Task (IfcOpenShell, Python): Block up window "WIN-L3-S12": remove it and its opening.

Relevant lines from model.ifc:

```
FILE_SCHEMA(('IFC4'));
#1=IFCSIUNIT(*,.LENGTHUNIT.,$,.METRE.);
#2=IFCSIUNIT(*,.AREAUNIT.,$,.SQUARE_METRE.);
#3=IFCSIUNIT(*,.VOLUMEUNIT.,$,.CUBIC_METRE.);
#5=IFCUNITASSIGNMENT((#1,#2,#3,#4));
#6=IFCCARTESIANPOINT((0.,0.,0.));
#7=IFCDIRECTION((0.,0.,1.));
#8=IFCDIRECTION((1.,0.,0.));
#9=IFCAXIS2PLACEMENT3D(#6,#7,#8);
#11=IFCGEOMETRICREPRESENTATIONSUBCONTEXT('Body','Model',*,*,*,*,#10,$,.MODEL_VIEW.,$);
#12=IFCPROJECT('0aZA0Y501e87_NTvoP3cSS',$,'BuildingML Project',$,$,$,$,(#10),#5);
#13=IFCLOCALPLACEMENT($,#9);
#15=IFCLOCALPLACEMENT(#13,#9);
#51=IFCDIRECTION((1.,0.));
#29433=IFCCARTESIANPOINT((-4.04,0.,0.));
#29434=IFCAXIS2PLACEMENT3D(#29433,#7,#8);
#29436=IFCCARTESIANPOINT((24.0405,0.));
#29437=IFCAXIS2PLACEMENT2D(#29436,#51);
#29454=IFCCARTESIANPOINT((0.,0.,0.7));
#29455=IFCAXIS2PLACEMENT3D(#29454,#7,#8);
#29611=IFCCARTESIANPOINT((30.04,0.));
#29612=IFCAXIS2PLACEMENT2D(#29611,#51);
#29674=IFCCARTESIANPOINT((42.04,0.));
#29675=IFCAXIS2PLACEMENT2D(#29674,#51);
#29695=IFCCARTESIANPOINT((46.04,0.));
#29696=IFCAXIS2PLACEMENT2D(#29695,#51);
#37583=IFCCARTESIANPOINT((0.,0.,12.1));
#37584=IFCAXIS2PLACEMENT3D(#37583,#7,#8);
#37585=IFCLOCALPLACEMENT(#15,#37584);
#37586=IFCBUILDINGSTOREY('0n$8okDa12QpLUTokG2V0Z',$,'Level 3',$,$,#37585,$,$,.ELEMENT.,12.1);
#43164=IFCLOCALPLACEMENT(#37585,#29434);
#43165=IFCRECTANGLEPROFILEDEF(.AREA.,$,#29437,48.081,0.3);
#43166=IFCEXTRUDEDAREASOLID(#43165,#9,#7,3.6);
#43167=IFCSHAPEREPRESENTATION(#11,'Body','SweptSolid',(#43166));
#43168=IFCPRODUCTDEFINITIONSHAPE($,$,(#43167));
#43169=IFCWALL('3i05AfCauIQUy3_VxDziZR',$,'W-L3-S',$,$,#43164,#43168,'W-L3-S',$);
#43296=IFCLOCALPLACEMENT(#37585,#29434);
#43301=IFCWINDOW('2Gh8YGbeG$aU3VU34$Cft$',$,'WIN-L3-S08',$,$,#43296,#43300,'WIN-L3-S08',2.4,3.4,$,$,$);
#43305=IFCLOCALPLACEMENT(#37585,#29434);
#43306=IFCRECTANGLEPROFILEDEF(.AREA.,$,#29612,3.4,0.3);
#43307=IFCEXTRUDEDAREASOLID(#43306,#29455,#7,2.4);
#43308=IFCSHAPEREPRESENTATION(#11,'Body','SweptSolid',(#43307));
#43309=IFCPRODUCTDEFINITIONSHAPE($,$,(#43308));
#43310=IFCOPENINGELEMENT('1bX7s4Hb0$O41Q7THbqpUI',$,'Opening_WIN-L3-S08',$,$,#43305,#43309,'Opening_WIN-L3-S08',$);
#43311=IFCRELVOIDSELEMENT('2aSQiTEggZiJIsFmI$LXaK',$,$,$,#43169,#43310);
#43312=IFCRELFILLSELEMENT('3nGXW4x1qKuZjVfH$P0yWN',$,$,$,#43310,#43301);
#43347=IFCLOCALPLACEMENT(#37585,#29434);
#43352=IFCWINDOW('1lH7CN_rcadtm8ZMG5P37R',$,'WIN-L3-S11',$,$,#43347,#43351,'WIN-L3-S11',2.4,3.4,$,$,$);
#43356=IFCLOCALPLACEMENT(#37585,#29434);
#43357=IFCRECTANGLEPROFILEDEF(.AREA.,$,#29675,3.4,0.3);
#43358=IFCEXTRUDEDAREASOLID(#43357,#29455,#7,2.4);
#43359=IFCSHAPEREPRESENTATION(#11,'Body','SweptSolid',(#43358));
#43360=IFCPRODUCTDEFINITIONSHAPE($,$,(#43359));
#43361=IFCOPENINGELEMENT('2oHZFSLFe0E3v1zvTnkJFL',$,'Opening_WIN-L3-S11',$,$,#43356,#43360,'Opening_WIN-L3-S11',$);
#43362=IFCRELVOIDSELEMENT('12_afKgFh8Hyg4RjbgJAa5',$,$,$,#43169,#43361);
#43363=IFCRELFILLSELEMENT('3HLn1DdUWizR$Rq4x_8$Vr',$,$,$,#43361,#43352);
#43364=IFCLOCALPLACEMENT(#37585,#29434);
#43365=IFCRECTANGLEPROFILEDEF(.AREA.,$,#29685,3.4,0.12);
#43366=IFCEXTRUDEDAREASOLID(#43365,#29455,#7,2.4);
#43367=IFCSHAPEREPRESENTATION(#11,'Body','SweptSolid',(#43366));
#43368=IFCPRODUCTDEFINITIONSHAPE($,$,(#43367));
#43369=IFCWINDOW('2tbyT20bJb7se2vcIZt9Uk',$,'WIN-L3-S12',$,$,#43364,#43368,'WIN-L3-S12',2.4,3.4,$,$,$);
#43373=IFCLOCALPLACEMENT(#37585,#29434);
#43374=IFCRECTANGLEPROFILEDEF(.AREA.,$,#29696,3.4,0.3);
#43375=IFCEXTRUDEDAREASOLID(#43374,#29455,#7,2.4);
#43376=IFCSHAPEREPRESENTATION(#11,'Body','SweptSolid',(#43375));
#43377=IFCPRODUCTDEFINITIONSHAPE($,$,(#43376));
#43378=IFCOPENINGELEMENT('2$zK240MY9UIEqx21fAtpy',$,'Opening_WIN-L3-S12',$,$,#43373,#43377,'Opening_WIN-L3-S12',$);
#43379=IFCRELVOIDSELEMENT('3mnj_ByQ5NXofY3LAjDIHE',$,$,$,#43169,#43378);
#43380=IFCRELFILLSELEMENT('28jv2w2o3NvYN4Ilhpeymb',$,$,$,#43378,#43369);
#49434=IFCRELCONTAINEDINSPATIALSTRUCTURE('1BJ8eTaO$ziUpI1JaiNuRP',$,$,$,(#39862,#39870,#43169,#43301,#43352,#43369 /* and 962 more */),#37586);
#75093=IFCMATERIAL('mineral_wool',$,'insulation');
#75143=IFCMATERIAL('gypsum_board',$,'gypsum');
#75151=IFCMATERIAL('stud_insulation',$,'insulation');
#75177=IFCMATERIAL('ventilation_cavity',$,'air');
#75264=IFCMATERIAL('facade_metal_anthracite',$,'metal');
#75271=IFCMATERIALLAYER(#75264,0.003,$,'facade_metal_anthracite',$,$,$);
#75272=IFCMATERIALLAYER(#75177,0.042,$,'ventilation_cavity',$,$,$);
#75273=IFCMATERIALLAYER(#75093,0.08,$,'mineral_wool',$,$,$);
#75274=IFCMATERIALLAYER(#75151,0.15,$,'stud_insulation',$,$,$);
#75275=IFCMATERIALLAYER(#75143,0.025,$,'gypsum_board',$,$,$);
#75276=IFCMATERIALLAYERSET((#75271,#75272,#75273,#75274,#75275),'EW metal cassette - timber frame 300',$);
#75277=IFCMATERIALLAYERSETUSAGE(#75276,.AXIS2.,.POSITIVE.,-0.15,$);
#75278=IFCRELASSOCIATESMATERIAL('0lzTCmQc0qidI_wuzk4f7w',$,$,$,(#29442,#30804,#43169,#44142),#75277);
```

```python
import ifcopenshell
import ifcopenshell.api.feature
import ifcopenshell.api.root
import ifcopenshell.geom
import ifcopenshell.util.shape

model = ifcopenshell.open("model.ifc")
settings = ifcopenshell.geom.settings()


def volume(element):
    """Net volume in cubic metres, openings subtracted."""
    shape = ifcopenshell.geom.create_shape(settings, element)
    return ifcopenshell.util.shape.get_volume(shape.geometry)


window = model.by_guid("2tbyT20bJb7se2vcIZt9Uk")
opening = window.FillsVoids[0].RelatingOpeningElement
wall = opening.VoidsElements[0].RelatingBuildingElement
before = volume(wall)

ifcopenshell.api.root.remove_product(model, product=window)
ifcopenshell.api.feature.remove_feature(model, feature=opening)

after = volume(wall)

print(f"wall volume {before:.3f} -> {after:.3f} m3")

model.write("model_v2.ifc")
```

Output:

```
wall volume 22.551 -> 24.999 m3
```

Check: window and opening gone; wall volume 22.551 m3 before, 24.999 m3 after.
